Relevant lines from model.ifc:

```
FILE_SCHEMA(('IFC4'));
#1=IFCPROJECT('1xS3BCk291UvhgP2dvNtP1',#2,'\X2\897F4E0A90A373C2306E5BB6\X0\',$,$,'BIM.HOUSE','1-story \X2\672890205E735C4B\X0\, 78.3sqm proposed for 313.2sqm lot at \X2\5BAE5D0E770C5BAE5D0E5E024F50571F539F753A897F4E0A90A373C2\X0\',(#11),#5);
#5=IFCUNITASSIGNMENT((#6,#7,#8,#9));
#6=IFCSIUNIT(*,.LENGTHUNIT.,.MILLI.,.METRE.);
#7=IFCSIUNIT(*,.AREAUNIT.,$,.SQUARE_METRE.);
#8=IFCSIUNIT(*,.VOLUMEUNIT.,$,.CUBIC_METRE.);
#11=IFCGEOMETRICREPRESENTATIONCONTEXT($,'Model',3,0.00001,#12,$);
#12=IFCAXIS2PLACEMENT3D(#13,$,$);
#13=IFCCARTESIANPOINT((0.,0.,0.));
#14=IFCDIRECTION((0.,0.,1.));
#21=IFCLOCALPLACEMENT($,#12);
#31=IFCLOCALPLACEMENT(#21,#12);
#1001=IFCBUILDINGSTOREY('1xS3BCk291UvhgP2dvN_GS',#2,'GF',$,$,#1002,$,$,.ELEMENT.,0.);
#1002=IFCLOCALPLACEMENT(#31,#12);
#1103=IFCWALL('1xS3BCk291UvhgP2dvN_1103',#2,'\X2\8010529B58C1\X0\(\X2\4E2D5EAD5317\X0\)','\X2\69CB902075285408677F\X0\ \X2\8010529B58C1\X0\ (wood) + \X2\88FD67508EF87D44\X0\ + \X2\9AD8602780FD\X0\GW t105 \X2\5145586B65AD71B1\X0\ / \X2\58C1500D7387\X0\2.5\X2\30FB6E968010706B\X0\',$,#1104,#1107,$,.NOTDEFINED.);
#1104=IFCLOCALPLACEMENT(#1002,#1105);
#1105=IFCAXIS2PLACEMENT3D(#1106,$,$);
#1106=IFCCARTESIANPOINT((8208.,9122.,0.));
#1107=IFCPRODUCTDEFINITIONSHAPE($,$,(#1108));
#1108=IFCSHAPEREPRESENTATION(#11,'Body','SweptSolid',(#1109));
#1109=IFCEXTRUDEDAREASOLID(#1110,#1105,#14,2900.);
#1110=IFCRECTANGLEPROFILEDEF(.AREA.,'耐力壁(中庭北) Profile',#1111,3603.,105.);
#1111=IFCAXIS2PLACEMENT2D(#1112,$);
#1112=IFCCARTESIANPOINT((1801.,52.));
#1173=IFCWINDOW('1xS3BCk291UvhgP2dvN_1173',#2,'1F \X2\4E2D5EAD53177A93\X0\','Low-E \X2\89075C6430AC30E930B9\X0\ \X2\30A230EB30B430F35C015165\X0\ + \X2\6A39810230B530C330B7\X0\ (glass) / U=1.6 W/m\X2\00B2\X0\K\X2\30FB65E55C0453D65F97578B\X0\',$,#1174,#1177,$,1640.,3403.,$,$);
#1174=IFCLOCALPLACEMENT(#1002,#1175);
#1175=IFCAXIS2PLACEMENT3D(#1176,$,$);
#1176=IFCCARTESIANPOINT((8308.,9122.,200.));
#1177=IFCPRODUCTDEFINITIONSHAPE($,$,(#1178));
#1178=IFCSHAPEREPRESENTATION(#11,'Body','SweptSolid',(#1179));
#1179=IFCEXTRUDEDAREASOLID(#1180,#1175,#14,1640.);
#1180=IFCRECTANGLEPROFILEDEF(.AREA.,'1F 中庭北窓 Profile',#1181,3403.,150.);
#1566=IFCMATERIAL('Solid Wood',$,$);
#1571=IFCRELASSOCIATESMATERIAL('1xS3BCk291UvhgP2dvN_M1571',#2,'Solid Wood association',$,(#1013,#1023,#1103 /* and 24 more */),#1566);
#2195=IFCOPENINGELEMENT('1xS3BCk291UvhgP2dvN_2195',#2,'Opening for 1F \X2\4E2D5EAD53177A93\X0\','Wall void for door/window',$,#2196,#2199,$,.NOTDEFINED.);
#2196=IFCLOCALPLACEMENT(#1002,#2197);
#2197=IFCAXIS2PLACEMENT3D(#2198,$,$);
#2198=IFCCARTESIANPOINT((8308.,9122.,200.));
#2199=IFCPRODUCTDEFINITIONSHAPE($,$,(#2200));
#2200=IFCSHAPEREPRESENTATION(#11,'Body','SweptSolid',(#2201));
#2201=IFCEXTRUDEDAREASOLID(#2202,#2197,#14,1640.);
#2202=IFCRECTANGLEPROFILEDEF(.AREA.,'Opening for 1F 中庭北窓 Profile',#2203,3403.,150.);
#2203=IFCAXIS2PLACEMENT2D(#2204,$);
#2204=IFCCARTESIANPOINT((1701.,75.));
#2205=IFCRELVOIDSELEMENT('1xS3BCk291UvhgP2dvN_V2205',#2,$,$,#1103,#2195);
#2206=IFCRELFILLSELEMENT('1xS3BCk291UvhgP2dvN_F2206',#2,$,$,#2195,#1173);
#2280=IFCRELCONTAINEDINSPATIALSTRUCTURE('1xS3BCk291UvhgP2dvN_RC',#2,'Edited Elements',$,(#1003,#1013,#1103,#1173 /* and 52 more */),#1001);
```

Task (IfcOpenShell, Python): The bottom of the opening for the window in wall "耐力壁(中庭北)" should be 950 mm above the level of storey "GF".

```python
import numpy as np
import ifcopenshell
import ifcopenshell.api.geometry
import ifcopenshell.geom
import ifcopenshell.util.element
import ifcopenshell.util.placement
import ifcopenshell.util.shape
import ifcopenshell.util.unit

model = ifcopenshell.open("model.ifc")
unit_scale = ifcopenshell.util.unit.calculate_unit_scale(model)

window = model.by_id(1173)
opening = window.FillsVoids[0].RelatingOpeningElement
storey = ifcopenshell.util.element.get_container(window, ifc_class="IfcBuildingStorey")
level = ifcopenshell.util.placement.get_local_placement(storey.ObjectPlacement)[2, 3]

# The opening's origin need not be at the sill, so measure its lowest point.
shape = ifcopenshell.geom.create_shape(ifcopenshell.geom.settings(), opening)
bottom = ifcopenshell.util.shape.get_shape_bottom_elevation(shape, shape.geometry) / unit_scale
dz = level + 0.95 / unit_scale - bottom

shift = np.array([0.0, 0.0, dz])
# The window is not placed relative to its opening, so move both.
for product in (opening, window):
    matrix = ifcopenshell.util.placement.get_local_placement(product.ObjectPlacement)
    matrix[:3, 3] += shift
    ifcopenshell.api.geometry.edit_object_placement(model, product=product, matrix=matrix, is_si=False)

print(f"moved by {dz * unit_scale:+.3f} m")

model.write("model-out.ifc")
```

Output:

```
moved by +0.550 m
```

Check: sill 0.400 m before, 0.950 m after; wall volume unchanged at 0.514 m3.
